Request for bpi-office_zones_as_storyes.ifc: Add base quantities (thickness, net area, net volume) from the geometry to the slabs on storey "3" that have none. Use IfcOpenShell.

First a look at what the model holds.

```python
import ifcopenshell
import ifcopenshell.util.element
import ifcopenshell.util.unit

model = ifcopenshell.open("bpi-office_zones_as_storyes.ifc")
print(model.schema)
for unit_type in ("LENGTHUNIT", "AREAUNIT", "VOLUMEUNIT"):
    print(unit_type, ifcopenshell.util.unit.calculate_unit_scale(model, unit_type))
storey = next(s for s in model.by_type("IfcBuildingStorey") if s.Name == "3")
slabs = [e for e in ifcopenshell.util.element.get_decomposition(storey) if e.is_a("IfcSlab")]
for e in sorted(slabs, key=lambda e: e.id()):
    print(e.id(), e.is_a(), e.Name, list(ifcopenshell.util.element.get_psets(e, qtos_only=True)), sep=" | ")
```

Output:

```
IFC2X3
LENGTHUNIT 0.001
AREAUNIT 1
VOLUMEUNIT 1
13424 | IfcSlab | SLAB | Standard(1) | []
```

```python
import ifcopenshell
import ifcopenshell.api.pset
import ifcopenshell.geom
import ifcopenshell.util.element
import ifcopenshell.util.shape
import ifcopenshell.util.unit

model = ifcopenshell.open("bpi-office_zones_as_storyes.ifc")
unit_scale = ifcopenshell.util.unit.calculate_unit_scale(model)
area_scale = ifcopenshell.util.unit.calculate_unit_scale(model, "AREAUNIT")
volume_scale = ifcopenshell.util.unit.calculate_unit_scale(model, "VOLUMEUNIT")
settings = ifcopenshell.geom.settings()

storey = next(s for s in model.by_type("IfcBuildingStorey") if s.Name == "3")
slabs = [e for e in ifcopenshell.util.element.get_decomposition(storey) if e.is_a("IfcSlab")]

for e in sorted(slabs, key=lambda e: e.id()):
    if ifcopenshell.util.element.get_psets(e, qtos_only=True, should_inherit=False):
        continue
    # Geometry comes back in metres, in the element's own axes.
    shape = ifcopenshell.geom.create_shape(settings, e)
    values = {
        "Width": ifcopenshell.util.shape.get_z(shape.geometry) / unit_scale,
        "NetArea": ifcopenshell.util.shape.get_footprint_area(shape.geometry) / area_scale,
        "NetVolume": ifcopenshell.util.shape.get_volume(shape.geometry) / volume_scale,
    }
    qto = ifcopenshell.api.pset.add_qto(model, product=e, name="BaseQuantities")
    ifcopenshell.api.pset.edit_qto(model, qto=qto, properties=values)
    print(e.id(), {k: round(v, 3) for k, v in values.items()})

model.write("bpi-office_zones_as_storyes_rev.ifc")
```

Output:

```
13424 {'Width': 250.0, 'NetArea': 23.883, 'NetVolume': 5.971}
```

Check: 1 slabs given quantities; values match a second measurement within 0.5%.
